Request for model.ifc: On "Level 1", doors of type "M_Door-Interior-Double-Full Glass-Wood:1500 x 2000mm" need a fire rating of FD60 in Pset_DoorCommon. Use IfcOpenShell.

First a look at what the model holds.

```python
import ifcopenshell
import ifcopenshell.util.element

model = ifcopenshell.open("model.ifc")
print(model.schema)
storey = next(s for s in model.by_type("IfcBuildingStorey") if s.Name == "Level 1")
doors = [e for e in ifcopenshell.util.element.get_decomposition(storey) if e.is_a("IfcDoor")]
seen = {}
for e in doors:
    element_type = ifcopenshell.util.element.get_type(e)
    key = (element_type.Name if element_type != e and element_type else None, ifcopenshell.util.element.get_pset(e, "Pset_DoorCommon", "FireRating"))
    seen[key] = seen.get(key, 0) + 1
for (name, value), count in sorted(seen.items(), key=str):
    print(count, "x", name, "|", value)
```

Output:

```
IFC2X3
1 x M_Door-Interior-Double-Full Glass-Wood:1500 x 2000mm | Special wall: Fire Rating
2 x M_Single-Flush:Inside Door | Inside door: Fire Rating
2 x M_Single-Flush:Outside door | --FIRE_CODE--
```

```python
import ifcopenshell
import ifcopenshell.api.pset
import ifcopenshell.util.element

model = ifcopenshell.open("model.ifc")

storey = next(s for s in model.by_type("IfcBuildingStorey") if s.Name == "Level 1")
doors = [e for e in ifcopenshell.util.element.get_decomposition(storey) if e.is_a("IfcDoor")]

count = 0
for e in doors:
    element_type = ifcopenshell.util.element.get_type(e)
    if element_type in (None, e) or element_type.Name != "M_Door-Interior-Double-Full Glass-Wood:1500 x 2000mm":
        continue
    # add_pset returns the element's existing set when there is one.
    pset = ifcopenshell.api.pset.add_pset(model, product=e, name="Pset_DoorCommon")
    ifcopenshell.api.pset.edit_pset(model, pset=pset, properties={"FireRating": "FD60"})
    count += 1

print(count, "doors updated")

model.write("model_updated.ifc")
```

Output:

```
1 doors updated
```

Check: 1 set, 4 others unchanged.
